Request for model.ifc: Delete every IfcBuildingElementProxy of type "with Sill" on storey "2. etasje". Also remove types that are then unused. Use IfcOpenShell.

First a look at what the model holds.

```python
import ifcopenshell
import ifcopenshell.util.element

model = ifcopenshell.open("model.ifc")
print(model.schema)
storey = next(s for s in model.by_type("IfcBuildingStorey") if s.Name == "2. etasje")
proxies = [e for e in ifcopenshell.util.element.get_decomposition(storey) if e.is_a("IfcBuildingElementProxy")]
seen = {}
for e in proxies:
    element_type = ifcopenshell.util.element.get_type(e)
    name = element_type.Name if element_type not in (None, e) else None
    seen[name] = seen.get(name, 0) + 1
for name, count in sorted(seen.items(), key=str):
    print(count, "x", name)
```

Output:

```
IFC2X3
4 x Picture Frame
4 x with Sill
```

```python
import ifcopenshell
import ifcopenshell.api.root
import ifcopenshell.util.element

model = ifcopenshell.open("model.ifc")

storey = next(s for s in model.by_type("IfcBuildingStorey") if s.Name == "2. etasje")
proxies = [e for e in ifcopenshell.util.element.get_decomposition(storey) if e.is_a("IfcBuildingElementProxy")]
targets = [e for e in proxies if (t := ifcopenshell.util.element.get_type(e)) not in (None, e) and t.Name == "with Sill"]
types = {ifcopenshell.util.element.get_type(e) for e in targets} - {None, *targets}

for e in targets:
    ifcopenshell.api.root.remove_product(model, product=e)
print(len(targets), "removed")

unused = [t for t in types if not ifcopenshell.util.element.get_types(t)]
for t in unused:
    ifcopenshell.api.root.remove_product(model, product=t)
print(len(unused), "unused types removed")

model.write("model_updated.ifc")
```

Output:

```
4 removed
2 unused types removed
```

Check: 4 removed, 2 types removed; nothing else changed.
